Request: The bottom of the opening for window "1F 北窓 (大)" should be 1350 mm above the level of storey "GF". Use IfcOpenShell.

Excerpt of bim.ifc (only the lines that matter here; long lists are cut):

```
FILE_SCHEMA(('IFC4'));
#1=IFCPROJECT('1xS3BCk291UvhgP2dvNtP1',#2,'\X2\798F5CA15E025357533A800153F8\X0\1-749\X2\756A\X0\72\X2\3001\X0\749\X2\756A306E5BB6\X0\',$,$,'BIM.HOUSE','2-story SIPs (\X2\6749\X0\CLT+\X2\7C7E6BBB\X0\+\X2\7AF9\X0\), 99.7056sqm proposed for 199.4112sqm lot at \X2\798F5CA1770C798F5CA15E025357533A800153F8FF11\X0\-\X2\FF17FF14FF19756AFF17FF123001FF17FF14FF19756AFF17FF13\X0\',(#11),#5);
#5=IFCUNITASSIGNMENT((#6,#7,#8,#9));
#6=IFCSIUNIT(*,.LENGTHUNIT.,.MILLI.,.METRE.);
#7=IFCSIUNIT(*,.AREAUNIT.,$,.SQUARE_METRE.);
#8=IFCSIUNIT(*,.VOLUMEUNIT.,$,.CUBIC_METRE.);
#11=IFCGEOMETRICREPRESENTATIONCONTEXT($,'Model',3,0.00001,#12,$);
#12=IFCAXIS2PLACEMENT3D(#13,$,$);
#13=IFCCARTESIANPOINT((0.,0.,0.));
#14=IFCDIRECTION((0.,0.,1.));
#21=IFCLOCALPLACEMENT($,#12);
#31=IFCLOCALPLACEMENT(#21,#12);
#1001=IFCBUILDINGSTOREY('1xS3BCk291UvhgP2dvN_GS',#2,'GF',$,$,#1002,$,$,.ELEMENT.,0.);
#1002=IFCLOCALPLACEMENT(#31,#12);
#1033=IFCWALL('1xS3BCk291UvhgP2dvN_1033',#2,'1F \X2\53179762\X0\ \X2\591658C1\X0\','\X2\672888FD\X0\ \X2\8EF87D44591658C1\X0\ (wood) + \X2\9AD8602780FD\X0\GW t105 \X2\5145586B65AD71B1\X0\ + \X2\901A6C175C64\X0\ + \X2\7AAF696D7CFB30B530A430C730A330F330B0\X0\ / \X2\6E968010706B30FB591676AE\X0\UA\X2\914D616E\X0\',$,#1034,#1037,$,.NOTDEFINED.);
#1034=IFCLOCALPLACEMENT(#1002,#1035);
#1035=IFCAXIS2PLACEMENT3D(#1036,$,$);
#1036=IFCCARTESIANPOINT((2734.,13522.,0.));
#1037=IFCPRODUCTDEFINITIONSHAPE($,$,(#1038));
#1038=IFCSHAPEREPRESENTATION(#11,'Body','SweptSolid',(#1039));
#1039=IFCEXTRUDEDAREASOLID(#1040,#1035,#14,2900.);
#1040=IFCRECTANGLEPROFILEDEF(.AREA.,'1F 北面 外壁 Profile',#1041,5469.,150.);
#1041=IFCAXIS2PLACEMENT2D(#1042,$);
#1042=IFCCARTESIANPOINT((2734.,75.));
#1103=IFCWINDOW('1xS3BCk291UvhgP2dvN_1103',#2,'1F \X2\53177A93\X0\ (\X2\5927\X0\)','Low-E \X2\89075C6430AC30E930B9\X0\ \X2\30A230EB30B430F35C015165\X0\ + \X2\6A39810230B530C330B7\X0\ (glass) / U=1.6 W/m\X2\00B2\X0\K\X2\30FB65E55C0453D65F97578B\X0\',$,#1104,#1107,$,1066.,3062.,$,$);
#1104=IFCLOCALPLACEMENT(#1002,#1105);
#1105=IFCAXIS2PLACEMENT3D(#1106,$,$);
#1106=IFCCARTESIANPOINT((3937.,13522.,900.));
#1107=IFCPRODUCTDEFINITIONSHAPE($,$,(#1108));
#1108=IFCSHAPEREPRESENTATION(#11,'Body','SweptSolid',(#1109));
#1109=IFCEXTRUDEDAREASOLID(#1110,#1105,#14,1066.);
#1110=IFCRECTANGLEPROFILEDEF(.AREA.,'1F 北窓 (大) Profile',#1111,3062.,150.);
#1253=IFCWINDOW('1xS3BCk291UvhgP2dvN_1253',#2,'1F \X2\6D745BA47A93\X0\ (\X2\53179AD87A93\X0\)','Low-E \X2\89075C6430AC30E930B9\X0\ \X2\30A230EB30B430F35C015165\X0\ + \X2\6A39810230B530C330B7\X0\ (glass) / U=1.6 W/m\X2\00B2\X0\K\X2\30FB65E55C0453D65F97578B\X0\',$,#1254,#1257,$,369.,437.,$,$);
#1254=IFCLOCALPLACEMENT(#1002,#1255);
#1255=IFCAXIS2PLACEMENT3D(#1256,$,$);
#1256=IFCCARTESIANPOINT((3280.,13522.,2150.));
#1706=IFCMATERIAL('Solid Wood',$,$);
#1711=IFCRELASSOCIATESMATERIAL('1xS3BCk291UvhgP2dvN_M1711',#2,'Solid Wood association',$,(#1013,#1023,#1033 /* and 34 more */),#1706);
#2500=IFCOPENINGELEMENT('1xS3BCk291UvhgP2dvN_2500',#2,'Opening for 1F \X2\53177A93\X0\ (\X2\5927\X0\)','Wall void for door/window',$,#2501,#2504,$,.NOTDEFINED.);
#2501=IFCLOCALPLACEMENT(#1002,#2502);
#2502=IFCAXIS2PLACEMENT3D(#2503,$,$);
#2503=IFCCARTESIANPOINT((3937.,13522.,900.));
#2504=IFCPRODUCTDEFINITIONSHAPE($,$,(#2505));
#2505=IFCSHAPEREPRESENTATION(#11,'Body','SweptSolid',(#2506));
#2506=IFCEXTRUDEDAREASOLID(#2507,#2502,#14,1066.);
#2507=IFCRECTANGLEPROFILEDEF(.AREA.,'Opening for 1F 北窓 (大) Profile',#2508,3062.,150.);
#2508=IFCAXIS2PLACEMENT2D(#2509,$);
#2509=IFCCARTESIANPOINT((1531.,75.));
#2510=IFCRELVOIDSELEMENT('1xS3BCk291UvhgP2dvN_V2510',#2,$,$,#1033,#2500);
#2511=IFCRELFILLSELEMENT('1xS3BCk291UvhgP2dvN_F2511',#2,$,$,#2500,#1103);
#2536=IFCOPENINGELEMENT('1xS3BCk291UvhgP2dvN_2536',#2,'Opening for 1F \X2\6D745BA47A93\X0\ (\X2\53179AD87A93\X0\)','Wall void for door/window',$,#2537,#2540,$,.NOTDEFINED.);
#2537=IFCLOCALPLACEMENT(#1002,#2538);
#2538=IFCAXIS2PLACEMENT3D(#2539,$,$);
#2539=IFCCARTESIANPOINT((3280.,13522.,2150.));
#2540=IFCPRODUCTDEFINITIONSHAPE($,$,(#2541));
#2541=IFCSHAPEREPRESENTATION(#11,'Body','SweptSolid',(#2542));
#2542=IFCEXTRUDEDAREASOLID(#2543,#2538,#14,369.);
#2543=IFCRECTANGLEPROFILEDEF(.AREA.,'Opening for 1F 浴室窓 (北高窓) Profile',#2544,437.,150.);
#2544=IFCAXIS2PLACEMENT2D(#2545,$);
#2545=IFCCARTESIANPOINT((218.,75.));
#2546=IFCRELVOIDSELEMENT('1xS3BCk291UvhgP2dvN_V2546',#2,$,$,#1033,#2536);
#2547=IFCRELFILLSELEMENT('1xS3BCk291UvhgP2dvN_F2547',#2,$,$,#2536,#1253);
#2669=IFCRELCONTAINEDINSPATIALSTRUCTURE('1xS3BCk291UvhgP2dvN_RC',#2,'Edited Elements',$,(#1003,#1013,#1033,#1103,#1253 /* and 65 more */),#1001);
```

```python
import numpy as np
import ifcopenshell
import ifcopenshell.api.geometry
import ifcopenshell.geom
import ifcopenshell.util.element
import ifcopenshell.util.placement
import ifcopenshell.util.shape
import ifcopenshell.util.unit

model = ifcopenshell.open("bim.ifc")
unit_scale = ifcopenshell.util.unit.calculate_unit_scale(model)

window = model.by_guid("1xS3BCk291UvhgP2dvN_1103")
opening = window.FillsVoids[0].RelatingOpeningElement
storey = ifcopenshell.util.element.get_container(window, ifc_class="IfcBuildingStorey")
level = ifcopenshell.util.placement.get_local_placement(storey.ObjectPlacement)[2, 3]

# The opening's origin need not be at the sill, so measure its lowest point.
shape = ifcopenshell.geom.create_shape(ifcopenshell.geom.settings(), opening)
bottom = ifcopenshell.util.shape.get_shape_bottom_elevation(shape, shape.geometry) / unit_scale
dz = level + 1350.0 - bottom

shift = np.array([0.0, 0.0, dz])
# The window is not placed relative to its opening, so move both.
for product in (opening, window):
    matrix = ifcopenshell.util.placement.get_local_placement(product.ObjectPlacement)
    matrix[:3, 3] += shift
    ifcopenshell.api.geometry.edit_object_placement(model, product=product, matrix=matrix, is_si=False)

print(f"moved by {dz * unit_scale:+.3f} m")

model.write("bim-out.ifc")
```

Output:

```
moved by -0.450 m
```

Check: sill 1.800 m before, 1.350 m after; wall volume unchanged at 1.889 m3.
